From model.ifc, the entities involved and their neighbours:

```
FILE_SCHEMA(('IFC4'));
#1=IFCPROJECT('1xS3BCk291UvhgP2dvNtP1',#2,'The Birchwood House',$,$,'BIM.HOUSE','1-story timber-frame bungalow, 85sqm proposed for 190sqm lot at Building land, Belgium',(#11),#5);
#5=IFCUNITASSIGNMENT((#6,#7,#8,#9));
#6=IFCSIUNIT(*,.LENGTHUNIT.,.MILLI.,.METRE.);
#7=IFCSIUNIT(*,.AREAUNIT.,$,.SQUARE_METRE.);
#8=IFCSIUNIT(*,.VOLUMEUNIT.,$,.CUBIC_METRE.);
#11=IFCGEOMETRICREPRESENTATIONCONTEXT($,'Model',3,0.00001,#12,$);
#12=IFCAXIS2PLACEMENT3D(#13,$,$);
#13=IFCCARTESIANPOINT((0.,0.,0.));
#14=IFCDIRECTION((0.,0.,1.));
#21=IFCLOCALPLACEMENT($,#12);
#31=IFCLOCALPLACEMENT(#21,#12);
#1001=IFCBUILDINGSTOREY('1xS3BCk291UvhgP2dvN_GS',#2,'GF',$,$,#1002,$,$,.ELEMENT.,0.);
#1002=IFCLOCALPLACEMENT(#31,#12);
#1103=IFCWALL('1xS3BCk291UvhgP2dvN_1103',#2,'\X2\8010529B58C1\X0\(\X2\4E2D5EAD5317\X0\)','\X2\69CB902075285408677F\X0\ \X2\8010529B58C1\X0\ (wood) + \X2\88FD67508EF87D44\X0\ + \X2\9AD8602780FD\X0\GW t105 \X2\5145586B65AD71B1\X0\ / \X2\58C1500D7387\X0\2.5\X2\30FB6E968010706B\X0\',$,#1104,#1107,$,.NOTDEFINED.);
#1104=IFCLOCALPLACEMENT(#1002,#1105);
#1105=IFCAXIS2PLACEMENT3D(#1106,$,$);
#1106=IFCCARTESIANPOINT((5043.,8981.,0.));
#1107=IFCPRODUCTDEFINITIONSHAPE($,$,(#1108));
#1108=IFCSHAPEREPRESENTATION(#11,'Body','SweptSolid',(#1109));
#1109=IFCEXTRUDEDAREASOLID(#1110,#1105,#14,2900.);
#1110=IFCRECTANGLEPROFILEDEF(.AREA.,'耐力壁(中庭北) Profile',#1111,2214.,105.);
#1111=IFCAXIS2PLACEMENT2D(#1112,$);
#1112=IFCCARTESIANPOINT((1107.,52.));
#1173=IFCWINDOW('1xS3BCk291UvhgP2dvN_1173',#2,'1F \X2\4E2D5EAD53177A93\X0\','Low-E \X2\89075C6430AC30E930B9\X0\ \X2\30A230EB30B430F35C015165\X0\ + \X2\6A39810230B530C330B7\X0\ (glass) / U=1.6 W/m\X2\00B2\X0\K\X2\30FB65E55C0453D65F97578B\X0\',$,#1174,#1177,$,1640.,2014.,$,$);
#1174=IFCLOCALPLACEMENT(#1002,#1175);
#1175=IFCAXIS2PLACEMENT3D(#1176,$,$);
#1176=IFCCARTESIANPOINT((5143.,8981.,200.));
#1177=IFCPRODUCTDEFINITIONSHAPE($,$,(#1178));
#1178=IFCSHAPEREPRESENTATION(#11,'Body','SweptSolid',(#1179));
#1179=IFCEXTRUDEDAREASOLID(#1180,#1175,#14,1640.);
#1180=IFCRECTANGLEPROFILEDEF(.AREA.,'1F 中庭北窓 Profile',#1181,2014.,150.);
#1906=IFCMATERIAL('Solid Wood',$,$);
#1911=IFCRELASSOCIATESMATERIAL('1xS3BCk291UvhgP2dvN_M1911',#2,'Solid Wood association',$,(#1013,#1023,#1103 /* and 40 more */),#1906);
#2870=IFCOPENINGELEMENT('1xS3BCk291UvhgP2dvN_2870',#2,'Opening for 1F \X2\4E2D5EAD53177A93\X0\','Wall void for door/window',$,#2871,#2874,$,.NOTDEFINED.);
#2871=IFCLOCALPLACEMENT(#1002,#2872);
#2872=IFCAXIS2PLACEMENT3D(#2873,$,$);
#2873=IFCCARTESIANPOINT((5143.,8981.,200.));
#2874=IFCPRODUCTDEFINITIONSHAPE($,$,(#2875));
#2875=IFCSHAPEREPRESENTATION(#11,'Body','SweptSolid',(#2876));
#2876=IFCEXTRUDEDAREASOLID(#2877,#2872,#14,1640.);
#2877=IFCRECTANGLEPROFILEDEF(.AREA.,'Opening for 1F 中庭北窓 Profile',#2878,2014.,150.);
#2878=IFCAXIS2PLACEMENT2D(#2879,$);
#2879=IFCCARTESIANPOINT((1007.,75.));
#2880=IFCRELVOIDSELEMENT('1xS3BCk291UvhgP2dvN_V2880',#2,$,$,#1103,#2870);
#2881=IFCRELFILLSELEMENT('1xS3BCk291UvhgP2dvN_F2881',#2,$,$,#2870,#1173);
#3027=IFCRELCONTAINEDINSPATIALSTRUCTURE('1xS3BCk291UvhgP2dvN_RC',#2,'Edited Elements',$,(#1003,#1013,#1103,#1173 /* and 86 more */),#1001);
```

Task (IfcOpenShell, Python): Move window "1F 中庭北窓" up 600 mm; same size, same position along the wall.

```python
import numpy as np
import ifcopenshell
import ifcopenshell.api.geometry
import ifcopenshell.util.placement
import ifcopenshell.util.unit

model = ifcopenshell.open("model.ifc")
unit_scale = ifcopenshell.util.unit.calculate_unit_scale(model)

window = model.by_guid("1xS3BCk291UvhgP2dvN_1173")
opening = window.FillsVoids[0].RelatingOpeningElement
dz = 0.6 / unit_scale

shift = np.array([0.0, 0.0, dz])
# The window is not placed relative to its opening, so move both.
for product in (opening, window):
    matrix = ifcopenshell.util.placement.get_local_placement(product.ObjectPlacement)
    matrix[:3, 3] += shift
    ifcopenshell.api.geometry.edit_object_placement(model, product=product, matrix=matrix, is_si=False)

print(f"moved by {dz * unit_scale:+.3f} m")

model.write("model_updated.ifc")
```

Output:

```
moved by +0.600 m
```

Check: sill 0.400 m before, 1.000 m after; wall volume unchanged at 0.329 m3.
